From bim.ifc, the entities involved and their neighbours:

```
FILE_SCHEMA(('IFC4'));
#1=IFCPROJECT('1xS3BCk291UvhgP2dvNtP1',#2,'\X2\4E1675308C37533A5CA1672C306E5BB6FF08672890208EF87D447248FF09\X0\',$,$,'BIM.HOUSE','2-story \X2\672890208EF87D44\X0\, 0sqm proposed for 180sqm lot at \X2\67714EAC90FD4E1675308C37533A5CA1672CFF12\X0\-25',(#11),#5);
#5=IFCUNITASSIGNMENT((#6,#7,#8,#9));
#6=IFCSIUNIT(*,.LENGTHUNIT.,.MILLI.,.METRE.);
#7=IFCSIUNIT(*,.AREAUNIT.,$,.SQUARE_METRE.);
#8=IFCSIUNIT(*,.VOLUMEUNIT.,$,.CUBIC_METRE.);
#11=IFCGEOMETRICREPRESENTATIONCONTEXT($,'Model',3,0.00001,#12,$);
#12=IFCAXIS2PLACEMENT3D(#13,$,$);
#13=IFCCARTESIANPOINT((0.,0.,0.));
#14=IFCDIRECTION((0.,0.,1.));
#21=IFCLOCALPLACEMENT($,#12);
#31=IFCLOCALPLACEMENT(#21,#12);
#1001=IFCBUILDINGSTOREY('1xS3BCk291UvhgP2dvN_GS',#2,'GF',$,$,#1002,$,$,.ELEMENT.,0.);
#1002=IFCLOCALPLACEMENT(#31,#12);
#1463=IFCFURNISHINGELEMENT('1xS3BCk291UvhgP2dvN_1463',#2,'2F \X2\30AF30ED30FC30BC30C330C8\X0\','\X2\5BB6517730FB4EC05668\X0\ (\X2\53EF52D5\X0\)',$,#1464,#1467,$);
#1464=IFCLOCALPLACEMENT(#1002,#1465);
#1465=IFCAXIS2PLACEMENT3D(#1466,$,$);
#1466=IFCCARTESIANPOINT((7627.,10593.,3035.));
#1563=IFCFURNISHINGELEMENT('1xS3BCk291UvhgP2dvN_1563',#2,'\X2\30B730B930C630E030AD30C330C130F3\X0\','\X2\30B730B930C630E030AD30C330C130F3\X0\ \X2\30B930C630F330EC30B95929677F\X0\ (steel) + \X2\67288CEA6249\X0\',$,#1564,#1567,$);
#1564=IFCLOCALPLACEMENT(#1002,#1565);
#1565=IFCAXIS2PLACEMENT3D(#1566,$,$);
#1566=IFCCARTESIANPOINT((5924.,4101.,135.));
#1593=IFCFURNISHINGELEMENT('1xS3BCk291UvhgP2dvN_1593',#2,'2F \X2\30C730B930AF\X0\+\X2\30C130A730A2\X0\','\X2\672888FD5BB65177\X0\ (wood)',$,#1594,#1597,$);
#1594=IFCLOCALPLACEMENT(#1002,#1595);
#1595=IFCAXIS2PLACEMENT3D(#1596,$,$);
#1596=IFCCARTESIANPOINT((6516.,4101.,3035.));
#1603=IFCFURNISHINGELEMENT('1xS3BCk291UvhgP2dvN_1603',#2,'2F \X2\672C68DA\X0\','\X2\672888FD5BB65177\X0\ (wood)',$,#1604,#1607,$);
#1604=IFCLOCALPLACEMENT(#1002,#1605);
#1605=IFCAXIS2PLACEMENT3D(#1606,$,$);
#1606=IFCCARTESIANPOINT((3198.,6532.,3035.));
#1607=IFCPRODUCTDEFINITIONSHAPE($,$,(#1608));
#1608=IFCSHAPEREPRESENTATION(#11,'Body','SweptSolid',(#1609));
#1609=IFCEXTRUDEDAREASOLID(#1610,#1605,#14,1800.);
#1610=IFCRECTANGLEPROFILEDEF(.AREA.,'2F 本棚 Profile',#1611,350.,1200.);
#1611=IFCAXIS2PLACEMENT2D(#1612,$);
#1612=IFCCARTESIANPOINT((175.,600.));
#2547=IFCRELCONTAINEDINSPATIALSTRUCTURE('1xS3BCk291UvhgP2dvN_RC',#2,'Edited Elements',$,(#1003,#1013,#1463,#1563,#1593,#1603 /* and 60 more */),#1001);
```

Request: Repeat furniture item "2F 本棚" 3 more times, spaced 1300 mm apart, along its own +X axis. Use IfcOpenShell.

```python
import ifcopenshell
import ifcopenshell.api.geometry
import ifcopenshell.api.root
import ifcopenshell.util.element
import ifcopenshell.util.placement
import ifcopenshell.util.unit

model = ifcopenshell.open("bim.ifc")
unit_scale = ifcopenshell.util.unit.calculate_unit_scale(model)


def reuse_history(source, copy):
    """copy_class also copies each property set's owner history, people and application; keep the originals."""
    for rel in copy.IsDefinedBy:
        if rel.is_a("IfcRelDefinesByProperties") and (history := rel.RelatingPropertyDefinition.OwnerHistory):
            rel.RelatingPropertyDefinition.OwnerHistory = source.OwnerHistory
            ifcopenshell.util.element.remove_deep2(model, history)


source = model.by_guid("1xS3BCk291UvhgP2dvN_1603")
base = ifcopenshell.util.placement.get_local_placement(source.ObjectPlacement)
step = base[:3, 0] * 1.3 / unit_scale

for i in range(1, 4):
    copy = ifcopenshell.api.root.copy_class(model, product=source)
    copy.Representation = ifcopenshell.util.element.copy_deep(
        model, source.Representation, exclude=["IfcGeometricRepresentationContext", "IfcRepresentationMap"]
    )
    reuse_history(source, copy)
    matrix = base.copy()
    matrix[:3, 3] += i * step
    print("added at", matrix[:3, 3].round(3) + 0.0)
    ifcopenshell.api.geometry.edit_object_placement(model, product=copy, matrix=matrix, is_si=False)

model.write("bim-out.ifc")
```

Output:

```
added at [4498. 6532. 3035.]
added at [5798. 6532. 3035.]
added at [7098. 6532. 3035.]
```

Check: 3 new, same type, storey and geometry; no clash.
